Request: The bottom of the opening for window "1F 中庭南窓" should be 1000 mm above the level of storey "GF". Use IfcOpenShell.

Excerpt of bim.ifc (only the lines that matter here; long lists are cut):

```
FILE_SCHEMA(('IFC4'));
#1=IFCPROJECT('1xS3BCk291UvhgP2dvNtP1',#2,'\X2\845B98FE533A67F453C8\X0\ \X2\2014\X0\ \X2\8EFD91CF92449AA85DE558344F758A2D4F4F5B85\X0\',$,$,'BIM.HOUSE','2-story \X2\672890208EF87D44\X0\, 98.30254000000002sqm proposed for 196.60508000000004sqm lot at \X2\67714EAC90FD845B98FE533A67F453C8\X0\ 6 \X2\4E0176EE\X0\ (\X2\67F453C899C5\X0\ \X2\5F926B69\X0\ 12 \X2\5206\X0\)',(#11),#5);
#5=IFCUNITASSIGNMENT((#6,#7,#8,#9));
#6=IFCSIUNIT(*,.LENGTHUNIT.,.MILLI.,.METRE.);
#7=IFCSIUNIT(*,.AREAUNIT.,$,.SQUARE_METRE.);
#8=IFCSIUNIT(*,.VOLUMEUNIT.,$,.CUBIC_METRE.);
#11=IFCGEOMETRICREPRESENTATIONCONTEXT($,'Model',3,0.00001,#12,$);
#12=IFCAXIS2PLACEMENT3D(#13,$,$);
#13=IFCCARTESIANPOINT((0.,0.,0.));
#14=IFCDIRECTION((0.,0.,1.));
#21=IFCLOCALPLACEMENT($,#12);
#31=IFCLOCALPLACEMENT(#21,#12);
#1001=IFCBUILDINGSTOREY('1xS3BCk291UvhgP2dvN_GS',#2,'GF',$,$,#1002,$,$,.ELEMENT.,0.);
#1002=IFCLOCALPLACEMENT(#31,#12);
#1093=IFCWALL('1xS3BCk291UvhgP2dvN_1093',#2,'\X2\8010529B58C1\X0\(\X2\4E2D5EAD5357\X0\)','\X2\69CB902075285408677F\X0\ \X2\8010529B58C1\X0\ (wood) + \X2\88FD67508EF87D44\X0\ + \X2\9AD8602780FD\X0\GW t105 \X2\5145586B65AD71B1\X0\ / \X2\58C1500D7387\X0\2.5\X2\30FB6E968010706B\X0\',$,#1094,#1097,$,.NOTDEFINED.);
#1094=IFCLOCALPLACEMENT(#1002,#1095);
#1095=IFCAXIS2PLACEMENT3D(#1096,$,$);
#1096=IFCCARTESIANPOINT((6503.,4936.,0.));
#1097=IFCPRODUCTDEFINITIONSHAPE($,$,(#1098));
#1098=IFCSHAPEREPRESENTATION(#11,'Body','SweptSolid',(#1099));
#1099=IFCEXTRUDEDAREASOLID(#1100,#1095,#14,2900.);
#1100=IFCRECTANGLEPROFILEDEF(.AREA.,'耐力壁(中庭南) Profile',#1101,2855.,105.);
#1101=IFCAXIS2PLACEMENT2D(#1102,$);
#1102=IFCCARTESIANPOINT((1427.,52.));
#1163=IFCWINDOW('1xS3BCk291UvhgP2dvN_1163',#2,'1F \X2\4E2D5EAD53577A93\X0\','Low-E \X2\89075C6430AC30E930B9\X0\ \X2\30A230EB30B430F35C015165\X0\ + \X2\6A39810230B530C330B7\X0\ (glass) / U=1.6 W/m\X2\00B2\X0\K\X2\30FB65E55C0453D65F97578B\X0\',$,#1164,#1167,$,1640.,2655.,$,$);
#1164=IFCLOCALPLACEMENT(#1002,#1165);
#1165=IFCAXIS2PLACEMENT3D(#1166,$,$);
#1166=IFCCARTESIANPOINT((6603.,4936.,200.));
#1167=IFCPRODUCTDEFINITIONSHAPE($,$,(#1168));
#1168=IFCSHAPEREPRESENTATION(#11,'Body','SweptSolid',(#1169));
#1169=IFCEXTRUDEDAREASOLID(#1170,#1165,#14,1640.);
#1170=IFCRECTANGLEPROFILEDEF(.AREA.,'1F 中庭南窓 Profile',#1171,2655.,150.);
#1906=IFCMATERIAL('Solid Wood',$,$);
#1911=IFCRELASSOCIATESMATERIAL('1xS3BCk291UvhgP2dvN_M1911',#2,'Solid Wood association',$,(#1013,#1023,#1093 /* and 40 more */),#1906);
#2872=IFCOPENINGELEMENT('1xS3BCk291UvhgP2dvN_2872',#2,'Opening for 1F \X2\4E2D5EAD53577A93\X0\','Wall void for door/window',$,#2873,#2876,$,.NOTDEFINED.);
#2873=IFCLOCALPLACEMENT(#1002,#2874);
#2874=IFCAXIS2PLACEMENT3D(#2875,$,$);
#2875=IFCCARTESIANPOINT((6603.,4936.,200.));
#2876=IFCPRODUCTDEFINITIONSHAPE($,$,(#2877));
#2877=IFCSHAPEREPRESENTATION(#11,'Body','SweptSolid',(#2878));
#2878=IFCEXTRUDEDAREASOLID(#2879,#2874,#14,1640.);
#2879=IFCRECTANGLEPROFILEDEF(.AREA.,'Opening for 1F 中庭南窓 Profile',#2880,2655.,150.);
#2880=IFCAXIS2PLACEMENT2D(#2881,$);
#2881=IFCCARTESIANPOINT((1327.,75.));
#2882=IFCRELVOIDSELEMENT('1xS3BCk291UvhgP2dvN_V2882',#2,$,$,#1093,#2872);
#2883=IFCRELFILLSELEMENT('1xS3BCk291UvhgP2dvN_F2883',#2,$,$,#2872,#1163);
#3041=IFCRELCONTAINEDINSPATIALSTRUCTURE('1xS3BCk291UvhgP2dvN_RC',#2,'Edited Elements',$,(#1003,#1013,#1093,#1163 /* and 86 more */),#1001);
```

```python
import numpy as np
import ifcopenshell
import ifcopenshell.api.geometry
import ifcopenshell.geom
import ifcopenshell.util.element
import ifcopenshell.util.placement
import ifcopenshell.util.shape
import ifcopenshell.util.unit

model = ifcopenshell.open("bim.ifc")
unit_scale = ifcopenshell.util.unit.calculate_unit_scale(model)

window = model.by_id(1163)
opening = window.FillsVoids[0].RelatingOpeningElement
storey = ifcopenshell.util.element.get_container(window, ifc_class="IfcBuildingStorey")
level = ifcopenshell.util.placement.get_local_placement(storey.ObjectPlacement)[2, 3]

# The opening's origin need not be at the sill, so measure its lowest point.
shape = ifcopenshell.geom.create_shape(ifcopenshell.geom.settings(), opening)
bottom = ifcopenshell.util.shape.get_shape_bottom_elevation(shape, shape.geometry) / unit_scale
dz = level + 1000.0 - bottom

shift = np.array([0.0, 0.0, dz])
# The window is not placed relative to its opening, so move both.
for product in (opening, window):
    matrix = ifcopenshell.util.placement.get_local_placement(product.ObjectPlacement)
    matrix[:3, 3] += shift
    ifcopenshell.api.geometry.edit_object_placement(model, product=product, matrix=matrix, is_si=False)

print(f"moved by {dz * unit_scale:+.3f} m")

model.write("bim_rev.ifc")
```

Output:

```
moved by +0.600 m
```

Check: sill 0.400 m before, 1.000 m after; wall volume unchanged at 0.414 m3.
